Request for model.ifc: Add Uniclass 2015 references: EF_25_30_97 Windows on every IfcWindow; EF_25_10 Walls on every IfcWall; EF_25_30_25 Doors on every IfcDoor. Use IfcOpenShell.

First a look at what the model holds.

```python
import ifcopenshell

model = ifcopenshell.open("model.ifc")
print(model.schema)
print("classifications:", [c.Name for c in model.by_type("IfcClassification")])
for ifc_class in ("IfcDoor", "IfcRoof", "IfcStair", "IfcWall", "IfcWindow"):
    print(ifc_class, len(model.by_type(ifc_class)))
```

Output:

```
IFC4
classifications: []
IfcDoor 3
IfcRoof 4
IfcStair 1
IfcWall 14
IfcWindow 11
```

```python
import ifcopenshell
import ifcopenshell.api.classification

model = ifcopenshell.open("model.ifc")

system = ifcopenshell.api.classification.add_classification(model, classification="Uniclass 2015")

codes = {
    "IfcWindow": ("EF_25_30_97", "Windows"),
    "IfcWall": ("EF_25_10", "Walls"),
    "IfcDoor": ("EF_25_30_25", "Doors"),
}
for ifc_class, (code, name) in codes.items():
    products = model.by_type(ifc_class)
    ifcopenshell.api.classification.add_reference(
        model, products=products, classification=system, identification=code, name=name
    )
    print(code, len(products))

model.write("model_updated.ifc")
```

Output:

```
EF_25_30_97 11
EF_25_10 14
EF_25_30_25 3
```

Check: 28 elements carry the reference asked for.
